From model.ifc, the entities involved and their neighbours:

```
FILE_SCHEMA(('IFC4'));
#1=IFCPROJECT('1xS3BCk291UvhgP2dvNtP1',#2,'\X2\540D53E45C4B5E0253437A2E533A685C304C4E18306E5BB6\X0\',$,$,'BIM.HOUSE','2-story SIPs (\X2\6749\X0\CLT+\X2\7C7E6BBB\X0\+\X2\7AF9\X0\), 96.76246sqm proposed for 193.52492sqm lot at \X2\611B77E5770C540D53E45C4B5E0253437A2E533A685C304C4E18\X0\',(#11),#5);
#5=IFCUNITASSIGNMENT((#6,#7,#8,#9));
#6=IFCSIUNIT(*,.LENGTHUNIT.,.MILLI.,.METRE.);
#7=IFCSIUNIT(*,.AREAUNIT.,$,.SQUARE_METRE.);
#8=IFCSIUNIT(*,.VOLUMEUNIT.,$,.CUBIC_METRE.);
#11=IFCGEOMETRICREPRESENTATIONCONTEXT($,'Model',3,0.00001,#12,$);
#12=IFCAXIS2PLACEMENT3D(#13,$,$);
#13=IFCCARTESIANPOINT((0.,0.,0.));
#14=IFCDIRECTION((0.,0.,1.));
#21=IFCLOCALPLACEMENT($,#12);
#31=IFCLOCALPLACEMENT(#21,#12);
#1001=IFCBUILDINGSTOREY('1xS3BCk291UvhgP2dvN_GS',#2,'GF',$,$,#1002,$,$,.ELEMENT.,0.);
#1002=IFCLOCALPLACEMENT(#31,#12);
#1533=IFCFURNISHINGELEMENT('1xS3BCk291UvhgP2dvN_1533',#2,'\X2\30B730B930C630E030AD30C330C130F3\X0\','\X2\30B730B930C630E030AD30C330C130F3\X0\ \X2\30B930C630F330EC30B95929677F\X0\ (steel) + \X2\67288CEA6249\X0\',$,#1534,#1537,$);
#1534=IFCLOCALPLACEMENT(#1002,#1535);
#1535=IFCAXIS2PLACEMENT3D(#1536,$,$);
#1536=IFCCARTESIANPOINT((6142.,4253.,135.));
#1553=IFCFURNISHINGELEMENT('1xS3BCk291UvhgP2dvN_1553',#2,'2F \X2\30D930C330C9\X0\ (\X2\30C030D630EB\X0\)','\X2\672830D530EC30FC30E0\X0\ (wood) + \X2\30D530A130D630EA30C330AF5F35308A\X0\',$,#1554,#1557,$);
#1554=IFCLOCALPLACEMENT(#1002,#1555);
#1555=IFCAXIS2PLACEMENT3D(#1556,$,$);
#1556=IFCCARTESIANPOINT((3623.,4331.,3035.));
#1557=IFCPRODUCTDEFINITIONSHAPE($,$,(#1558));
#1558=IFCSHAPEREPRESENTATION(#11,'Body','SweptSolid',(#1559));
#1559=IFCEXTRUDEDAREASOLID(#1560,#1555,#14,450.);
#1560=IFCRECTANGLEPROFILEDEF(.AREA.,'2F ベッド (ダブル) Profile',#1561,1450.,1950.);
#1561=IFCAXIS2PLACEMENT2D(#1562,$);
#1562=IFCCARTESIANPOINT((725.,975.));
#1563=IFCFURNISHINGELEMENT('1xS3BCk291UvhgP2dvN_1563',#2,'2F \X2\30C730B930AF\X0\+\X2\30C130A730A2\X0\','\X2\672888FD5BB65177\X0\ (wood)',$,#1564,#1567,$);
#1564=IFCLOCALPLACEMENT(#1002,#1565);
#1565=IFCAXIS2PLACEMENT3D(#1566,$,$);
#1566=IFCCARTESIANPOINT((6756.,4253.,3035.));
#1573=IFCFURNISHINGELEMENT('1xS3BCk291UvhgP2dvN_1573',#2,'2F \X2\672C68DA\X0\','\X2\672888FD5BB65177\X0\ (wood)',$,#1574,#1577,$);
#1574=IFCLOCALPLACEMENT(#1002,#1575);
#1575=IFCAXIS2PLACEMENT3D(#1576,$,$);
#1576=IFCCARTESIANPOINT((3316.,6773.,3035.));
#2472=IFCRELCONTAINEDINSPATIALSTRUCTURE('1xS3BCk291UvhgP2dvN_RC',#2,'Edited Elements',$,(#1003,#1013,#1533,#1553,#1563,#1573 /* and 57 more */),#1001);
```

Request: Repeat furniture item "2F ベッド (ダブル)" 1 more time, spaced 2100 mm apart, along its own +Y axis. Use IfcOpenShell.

```python
import ifcopenshell
import ifcopenshell.api.geometry
import ifcopenshell.api.root
import ifcopenshell.util.element
import ifcopenshell.util.placement
import ifcopenshell.util.unit

model = ifcopenshell.open("model.ifc")
unit_scale = ifcopenshell.util.unit.calculate_unit_scale(model)


def reuse_history(source, copy):
    """copy_class also copies each property set's owner history, people and application; keep the originals."""
    for rel in copy.IsDefinedBy:
        if rel.is_a("IfcRelDefinesByProperties") and (history := rel.RelatingPropertyDefinition.OwnerHistory):
            rel.RelatingPropertyDefinition.OwnerHistory = source.OwnerHistory
            ifcopenshell.util.element.remove_deep2(model, history)


source = model.by_id(1553)
base = ifcopenshell.util.placement.get_local_placement(source.ObjectPlacement)
step = base[:3, 1] * 2.1 / unit_scale

for i in range(1, 2):
    copy = ifcopenshell.api.root.copy_class(model, product=source)
    copy.Representation = ifcopenshell.util.element.copy_deep(
        model, source.Representation, exclude=["IfcGeometricRepresentationContext", "IfcRepresentationMap"]
    )
    reuse_history(source, copy)
    matrix = base.copy()
    matrix[:3, 3] += i * step
    print("added at", matrix[:3, 3].round(3) + 0.0)
    ifcopenshell.api.geometry.edit_object_placement(model, product=copy, matrix=matrix, is_si=False)

model.write("model_rev.ifc")
```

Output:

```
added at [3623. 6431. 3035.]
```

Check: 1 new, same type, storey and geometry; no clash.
